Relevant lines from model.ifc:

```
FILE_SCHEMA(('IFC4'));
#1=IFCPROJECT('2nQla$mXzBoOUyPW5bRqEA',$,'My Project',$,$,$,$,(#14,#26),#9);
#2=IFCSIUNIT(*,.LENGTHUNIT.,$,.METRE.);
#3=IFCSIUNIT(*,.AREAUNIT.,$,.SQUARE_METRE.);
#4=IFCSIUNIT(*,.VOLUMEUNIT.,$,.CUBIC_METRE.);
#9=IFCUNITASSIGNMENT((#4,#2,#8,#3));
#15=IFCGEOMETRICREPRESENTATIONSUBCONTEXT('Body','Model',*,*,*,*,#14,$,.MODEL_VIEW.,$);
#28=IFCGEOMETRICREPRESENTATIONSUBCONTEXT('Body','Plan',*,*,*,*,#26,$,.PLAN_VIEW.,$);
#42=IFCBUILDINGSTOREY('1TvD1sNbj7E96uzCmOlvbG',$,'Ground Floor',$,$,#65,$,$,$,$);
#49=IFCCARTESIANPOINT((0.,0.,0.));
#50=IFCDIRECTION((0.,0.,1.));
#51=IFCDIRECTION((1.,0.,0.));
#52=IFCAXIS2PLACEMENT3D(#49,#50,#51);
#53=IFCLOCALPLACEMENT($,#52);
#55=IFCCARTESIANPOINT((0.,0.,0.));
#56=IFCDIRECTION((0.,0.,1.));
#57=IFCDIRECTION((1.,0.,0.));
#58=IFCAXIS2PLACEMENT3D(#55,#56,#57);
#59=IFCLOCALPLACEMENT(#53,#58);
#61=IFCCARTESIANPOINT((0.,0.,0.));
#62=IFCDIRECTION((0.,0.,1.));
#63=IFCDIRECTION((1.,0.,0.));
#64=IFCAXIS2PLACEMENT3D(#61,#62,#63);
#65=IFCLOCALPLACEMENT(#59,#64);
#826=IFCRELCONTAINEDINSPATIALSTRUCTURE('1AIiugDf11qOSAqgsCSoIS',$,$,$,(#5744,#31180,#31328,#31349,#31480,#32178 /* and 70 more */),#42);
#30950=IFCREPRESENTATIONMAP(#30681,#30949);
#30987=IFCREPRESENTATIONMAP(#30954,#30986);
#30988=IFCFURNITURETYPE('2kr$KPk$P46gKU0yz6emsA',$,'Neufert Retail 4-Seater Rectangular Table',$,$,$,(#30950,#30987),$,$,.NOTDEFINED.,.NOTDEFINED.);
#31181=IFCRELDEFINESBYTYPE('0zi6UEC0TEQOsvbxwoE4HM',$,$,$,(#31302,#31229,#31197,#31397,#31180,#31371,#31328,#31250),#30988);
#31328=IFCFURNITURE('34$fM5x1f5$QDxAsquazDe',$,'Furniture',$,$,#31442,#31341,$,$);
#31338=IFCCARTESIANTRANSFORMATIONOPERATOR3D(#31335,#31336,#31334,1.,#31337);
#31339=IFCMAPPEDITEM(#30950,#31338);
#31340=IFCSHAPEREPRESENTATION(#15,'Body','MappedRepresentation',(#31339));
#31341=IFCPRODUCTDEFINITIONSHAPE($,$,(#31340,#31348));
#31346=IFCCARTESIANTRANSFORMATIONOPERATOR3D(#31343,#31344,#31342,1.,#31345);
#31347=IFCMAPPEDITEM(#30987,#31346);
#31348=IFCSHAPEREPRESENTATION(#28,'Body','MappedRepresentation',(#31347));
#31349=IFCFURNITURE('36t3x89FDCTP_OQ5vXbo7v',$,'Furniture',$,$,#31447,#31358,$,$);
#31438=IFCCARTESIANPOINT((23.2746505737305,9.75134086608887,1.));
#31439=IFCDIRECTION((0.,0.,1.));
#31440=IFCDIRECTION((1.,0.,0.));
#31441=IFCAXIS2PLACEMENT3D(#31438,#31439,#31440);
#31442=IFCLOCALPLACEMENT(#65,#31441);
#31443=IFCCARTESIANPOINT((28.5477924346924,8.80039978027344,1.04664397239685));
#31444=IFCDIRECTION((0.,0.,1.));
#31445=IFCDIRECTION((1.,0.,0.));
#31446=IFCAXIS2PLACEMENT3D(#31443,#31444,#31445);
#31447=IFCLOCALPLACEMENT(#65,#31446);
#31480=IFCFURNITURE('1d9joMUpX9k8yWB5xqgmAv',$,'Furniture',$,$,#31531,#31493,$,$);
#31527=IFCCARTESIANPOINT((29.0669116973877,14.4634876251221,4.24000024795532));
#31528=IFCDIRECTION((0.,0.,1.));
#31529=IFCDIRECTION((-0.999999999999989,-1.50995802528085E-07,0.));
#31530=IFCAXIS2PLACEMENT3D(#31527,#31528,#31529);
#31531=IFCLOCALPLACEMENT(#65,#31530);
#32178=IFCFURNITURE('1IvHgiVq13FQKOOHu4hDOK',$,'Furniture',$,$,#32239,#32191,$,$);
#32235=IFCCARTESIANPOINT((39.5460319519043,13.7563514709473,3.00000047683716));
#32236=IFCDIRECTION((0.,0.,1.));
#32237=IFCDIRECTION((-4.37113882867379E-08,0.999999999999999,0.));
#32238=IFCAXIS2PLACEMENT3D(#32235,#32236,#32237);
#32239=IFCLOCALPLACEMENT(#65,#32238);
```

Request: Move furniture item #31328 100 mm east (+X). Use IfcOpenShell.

```python
import ifcopenshell
import ifcopenshell.api.geometry
import ifcopenshell.util.placement
import ifcopenshell.util.unit

model = ifcopenshell.open("model.ifc")
unit_scale = ifcopenshell.util.unit.calculate_unit_scale(model)

item = model.by_id(31328)
matrix = ifcopenshell.util.placement.get_local_placement(item.ObjectPlacement)
matrix[0, 3] += 0.1 / unit_scale
ifcopenshell.api.geometry.edit_object_placement(model, product=item, matrix=matrix, is_si=False)

print(ifcopenshell.util.placement.get_local_placement(item.ObjectPlacement).round(3) + 0.0)

model.write("model_edited.ifc")
```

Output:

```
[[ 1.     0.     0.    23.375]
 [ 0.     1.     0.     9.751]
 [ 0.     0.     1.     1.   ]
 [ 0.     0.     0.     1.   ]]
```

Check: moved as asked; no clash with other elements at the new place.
